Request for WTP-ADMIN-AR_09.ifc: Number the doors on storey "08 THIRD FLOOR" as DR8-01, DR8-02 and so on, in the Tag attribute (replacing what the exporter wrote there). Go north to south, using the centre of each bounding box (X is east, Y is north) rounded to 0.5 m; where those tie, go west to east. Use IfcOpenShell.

First a look at what the model holds.

```python
import ifcopenshell
import ifcopenshell.util.element
import ifcopenshell.util.placement

model = ifcopenshell.open("WTP-ADMIN-AR_09.ifc")
print(model.schema)
storey = next(s for s in model.by_type("IfcBuildingStorey") if s.Name == "08 THIRD FLOOR")
doors = [e for e in ifcopenshell.util.element.get_decomposition(storey) if e.is_a("IfcDoor")]
for e in sorted(doors, key=lambda e: e.id()):
    origin = ifcopenshell.util.placement.get_local_placement(e.ObjectPlacement)[:3, 3]
    print(e.id(), e.Tag, e.Name, origin.round(2) + 0.0, sep=" | ")
```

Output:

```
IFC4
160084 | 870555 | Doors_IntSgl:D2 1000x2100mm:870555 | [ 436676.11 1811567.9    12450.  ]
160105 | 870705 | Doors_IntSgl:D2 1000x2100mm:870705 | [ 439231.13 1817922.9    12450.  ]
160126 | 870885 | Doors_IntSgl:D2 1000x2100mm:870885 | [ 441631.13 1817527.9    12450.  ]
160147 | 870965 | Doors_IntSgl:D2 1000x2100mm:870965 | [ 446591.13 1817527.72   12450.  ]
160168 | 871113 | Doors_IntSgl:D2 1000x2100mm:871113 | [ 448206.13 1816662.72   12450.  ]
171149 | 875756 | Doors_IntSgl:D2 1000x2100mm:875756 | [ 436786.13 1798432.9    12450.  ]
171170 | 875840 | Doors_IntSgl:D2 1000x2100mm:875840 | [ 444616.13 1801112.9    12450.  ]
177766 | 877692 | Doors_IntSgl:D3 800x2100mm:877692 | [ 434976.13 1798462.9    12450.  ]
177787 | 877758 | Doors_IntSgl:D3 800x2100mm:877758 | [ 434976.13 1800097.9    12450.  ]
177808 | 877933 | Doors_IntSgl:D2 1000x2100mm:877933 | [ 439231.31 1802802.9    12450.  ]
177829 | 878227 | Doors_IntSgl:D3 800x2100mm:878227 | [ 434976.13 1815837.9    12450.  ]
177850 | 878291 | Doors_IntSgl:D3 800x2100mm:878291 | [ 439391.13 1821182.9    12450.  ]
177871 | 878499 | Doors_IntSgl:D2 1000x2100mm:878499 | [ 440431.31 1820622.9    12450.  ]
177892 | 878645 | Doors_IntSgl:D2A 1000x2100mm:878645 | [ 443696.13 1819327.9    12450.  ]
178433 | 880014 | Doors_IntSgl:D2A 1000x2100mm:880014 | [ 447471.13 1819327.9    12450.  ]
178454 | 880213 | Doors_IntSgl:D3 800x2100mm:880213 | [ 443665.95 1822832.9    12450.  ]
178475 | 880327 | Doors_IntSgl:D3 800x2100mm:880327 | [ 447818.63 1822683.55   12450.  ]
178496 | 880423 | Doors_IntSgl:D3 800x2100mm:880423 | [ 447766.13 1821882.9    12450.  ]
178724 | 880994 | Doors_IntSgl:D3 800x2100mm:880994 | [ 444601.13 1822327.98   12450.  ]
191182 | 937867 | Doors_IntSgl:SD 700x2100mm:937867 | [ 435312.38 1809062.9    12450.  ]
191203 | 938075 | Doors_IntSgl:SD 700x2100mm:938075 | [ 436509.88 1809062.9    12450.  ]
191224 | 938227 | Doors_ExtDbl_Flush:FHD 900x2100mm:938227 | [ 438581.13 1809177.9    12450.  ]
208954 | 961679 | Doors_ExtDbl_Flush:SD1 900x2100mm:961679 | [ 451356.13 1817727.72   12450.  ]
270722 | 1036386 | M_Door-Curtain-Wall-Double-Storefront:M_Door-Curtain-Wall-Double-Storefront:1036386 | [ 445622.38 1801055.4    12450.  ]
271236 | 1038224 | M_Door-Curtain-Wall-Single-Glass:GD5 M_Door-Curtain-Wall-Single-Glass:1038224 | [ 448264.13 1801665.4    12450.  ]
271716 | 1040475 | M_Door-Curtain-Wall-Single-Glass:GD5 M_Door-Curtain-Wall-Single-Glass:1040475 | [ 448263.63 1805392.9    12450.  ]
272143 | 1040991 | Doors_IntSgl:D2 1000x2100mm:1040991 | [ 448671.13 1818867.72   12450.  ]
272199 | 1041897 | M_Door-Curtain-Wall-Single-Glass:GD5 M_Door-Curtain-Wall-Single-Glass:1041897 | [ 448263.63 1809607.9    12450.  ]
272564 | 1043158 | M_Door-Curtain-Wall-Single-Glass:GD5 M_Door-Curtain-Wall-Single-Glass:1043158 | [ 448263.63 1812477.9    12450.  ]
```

```python
import ifcopenshell
import ifcopenshell.geom
import ifcopenshell.util.element
import ifcopenshell.util.shape

model = ifcopenshell.open("WTP-ADMIN-AR_09.ifc")
settings = ifcopenshell.geom.settings()
settings.set("use-world-coords", True)


def centre(element):
    shape = ifcopenshell.geom.create_shape(settings, element)
    return ifcopenshell.util.shape.get_bbox_centroid(shape.geometry)


storey = next(s for s in model.by_type("IfcBuildingStorey") if s.Name == "08 THIRD FLOOR")
doors = [e for e in ifcopenshell.util.element.get_decomposition(storey) if e.is_a("IfcDoor")]

# Insertion points can sit at a corner or the storey origin, so sort by the geometry (in metres).
centres = {e: centre(e) for e in doors}
doors.sort(key=lambda e: (-round(centres[e][1] / 0.5), centres[e][0]))

for i, e in enumerate(doors, start=1):
    number = f"DR8-{i:02d}"
    e.Tag = number
    print(e.id(), number)

model.write("WTP-ADMIN-AR_09_rev.ifc")
```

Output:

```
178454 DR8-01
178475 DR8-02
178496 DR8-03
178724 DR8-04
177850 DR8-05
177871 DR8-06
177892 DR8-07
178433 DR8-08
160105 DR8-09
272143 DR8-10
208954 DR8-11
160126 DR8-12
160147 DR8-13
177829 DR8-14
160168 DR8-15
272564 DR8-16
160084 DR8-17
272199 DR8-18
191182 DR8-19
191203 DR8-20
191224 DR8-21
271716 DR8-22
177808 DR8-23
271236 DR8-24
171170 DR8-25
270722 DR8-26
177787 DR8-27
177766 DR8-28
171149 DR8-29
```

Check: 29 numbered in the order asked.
